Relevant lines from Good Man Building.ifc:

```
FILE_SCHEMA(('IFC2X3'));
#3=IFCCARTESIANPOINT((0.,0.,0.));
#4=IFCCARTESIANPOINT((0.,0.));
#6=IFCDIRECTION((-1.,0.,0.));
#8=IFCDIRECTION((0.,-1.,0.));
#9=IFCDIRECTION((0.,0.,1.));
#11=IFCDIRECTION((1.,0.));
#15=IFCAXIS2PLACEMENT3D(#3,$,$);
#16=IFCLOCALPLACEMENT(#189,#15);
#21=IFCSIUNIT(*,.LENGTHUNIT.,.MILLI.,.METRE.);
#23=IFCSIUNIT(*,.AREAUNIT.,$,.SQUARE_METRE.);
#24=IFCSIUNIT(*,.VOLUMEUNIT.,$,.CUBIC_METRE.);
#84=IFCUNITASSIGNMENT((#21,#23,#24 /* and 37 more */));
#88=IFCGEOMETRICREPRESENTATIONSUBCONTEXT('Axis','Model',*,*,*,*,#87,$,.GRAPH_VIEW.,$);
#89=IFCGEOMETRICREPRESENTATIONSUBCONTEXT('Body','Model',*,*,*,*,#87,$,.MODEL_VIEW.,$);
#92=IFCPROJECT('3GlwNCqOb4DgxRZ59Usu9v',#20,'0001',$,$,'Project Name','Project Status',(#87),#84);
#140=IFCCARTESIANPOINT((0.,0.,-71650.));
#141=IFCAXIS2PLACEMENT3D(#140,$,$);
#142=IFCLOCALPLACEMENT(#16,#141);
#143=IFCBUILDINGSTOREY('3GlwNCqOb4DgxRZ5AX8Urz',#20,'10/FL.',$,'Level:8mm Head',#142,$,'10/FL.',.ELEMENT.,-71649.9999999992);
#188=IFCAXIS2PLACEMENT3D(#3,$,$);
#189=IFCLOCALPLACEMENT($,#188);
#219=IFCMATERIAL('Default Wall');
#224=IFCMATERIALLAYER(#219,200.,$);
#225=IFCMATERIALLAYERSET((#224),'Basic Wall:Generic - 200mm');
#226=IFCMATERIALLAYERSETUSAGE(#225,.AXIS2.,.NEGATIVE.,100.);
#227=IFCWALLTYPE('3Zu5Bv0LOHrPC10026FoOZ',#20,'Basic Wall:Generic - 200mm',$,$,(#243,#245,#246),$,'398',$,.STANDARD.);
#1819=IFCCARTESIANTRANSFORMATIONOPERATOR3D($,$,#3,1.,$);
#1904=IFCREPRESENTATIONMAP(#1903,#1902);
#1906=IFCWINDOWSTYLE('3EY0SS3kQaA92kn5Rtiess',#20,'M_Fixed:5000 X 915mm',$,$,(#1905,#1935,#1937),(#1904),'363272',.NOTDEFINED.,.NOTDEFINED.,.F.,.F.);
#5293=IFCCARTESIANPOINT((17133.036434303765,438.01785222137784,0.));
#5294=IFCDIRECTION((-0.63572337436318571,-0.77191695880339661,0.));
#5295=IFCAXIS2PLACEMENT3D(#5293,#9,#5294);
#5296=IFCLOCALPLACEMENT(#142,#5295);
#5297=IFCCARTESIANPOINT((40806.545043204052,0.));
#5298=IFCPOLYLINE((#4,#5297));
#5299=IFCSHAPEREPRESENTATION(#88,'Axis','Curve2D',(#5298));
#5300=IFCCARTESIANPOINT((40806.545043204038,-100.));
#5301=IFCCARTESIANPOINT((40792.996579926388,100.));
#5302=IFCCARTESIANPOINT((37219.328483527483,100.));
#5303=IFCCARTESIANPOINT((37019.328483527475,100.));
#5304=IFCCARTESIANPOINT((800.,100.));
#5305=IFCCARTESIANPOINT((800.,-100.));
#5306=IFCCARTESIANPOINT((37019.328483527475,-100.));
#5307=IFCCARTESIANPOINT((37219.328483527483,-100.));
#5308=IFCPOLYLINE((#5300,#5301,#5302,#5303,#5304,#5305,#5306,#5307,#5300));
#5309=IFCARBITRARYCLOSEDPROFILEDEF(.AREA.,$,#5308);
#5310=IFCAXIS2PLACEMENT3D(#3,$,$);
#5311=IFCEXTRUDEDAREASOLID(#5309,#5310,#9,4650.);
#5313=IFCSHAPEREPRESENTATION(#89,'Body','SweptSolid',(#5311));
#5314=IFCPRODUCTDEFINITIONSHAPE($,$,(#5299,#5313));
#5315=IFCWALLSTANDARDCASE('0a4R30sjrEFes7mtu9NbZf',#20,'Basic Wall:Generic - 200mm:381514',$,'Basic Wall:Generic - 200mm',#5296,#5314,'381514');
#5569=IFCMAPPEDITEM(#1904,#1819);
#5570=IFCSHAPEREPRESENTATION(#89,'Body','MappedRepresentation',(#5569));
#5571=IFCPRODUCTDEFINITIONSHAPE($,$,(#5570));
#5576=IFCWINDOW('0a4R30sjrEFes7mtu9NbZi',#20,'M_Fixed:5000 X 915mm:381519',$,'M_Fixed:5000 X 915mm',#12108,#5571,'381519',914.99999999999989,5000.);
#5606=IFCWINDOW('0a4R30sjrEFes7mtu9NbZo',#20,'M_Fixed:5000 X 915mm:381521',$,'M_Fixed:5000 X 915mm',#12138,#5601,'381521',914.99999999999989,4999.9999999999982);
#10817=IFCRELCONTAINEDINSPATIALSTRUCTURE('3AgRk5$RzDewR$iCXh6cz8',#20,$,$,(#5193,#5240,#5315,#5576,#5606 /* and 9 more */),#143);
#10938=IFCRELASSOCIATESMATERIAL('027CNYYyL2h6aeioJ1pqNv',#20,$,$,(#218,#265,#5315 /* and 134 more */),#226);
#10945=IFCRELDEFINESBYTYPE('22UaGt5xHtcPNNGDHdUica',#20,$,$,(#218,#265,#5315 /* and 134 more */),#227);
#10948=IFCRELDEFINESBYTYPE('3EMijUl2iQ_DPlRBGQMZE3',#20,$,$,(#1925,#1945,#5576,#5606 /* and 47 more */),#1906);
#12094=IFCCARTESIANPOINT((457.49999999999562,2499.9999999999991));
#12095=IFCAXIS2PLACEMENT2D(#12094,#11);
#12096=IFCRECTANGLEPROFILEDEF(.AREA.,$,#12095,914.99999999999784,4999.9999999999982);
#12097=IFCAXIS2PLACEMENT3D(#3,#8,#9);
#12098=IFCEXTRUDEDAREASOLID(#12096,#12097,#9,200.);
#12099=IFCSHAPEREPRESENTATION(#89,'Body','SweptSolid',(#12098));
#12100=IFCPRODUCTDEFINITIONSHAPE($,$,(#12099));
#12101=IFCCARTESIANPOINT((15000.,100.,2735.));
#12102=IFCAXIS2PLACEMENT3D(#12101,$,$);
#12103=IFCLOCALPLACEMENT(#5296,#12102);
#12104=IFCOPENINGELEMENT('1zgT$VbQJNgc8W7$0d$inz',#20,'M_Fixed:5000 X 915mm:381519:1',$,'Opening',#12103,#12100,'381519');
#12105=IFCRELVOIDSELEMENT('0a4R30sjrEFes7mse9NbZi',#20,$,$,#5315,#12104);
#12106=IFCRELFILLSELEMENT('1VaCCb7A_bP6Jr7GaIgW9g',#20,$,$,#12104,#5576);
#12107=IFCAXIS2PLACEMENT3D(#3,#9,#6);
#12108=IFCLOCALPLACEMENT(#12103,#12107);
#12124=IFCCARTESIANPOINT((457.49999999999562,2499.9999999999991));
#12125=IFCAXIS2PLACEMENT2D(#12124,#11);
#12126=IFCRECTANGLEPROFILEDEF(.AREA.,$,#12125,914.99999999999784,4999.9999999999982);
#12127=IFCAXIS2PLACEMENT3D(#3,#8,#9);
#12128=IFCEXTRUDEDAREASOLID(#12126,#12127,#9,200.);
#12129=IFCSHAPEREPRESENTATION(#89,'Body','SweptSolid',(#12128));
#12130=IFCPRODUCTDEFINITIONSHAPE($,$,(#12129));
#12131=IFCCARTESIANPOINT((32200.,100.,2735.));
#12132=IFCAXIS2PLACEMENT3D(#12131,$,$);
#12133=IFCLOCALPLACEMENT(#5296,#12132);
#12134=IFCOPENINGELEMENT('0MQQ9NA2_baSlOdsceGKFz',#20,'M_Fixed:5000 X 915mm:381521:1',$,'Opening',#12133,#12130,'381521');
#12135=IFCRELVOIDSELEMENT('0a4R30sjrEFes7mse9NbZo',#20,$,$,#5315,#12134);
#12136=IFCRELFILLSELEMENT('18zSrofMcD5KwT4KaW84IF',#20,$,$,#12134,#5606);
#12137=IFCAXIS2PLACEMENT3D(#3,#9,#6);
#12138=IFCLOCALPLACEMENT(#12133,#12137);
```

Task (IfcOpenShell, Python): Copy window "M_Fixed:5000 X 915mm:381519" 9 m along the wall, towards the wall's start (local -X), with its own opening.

```python
import ifcopenshell
import ifcopenshell.api.feature
import ifcopenshell.api.geometry
import ifcopenshell.api.root
import ifcopenshell.geom
import ifcopenshell.util.element
import ifcopenshell.util.placement
import ifcopenshell.util.shape
import ifcopenshell.util.unit

model = ifcopenshell.open("Good Man Building.ifc")
unit_scale = ifcopenshell.util.unit.calculate_unit_scale(model)
settings = ifcopenshell.geom.settings()


def volume(element):
    """Net volume in cubic metres, openings subtracted."""
    shape = ifcopenshell.geom.create_shape(settings, element)
    return ifcopenshell.util.shape.get_volume(shape.geometry)


def reuse_history(source, copy):
    """copy_class also copies each property set's owner history, people and application; keep the originals."""
    for rel in copy.IsDefinedBy:
        if rel.is_a("IfcRelDefinesByProperties") and (history := rel.RelatingPropertyDefinition.OwnerHistory):
            rel.RelatingPropertyDefinition.OwnerHistory = source.OwnerHistory
            ifcopenshell.util.element.remove_deep2(model, history)


window = model.by_id(5576)
opening = window.FillsVoids[0].RelatingOpeningElement
wall = opening.VoidsElements[0].RelatingBuildingElement
before = volume(wall)
shift = ifcopenshell.util.placement.get_local_placement(wall.ObjectPlacement)[:3, 0] * -9 / unit_scale

# copy_class copies the void relationship, type, container and properties, but no geometry.
new_opening = ifcopenshell.api.root.copy_class(model, product=opening)
new_opening.Representation = ifcopenshell.util.element.copy_deep(
    model, opening.Representation, exclude=["IfcGeometricRepresentationContext", "IfcRepresentationMap"]
)
new_opening.Name = "M_Fixed:5000 X 915mm"
new_opening.Tag = None
new_window = ifcopenshell.api.root.copy_class(model, product=window)
new_window.Representation = ifcopenshell.util.element.copy_deep(
    model, window.Representation, exclude=["IfcGeometricRepresentationContext", "IfcRepresentationMap"]
)
new_window.Name = "M_Fixed:5000 X 915mm"
new_window.Tag = None
reuse_history(window, new_window)
fills = ifcopenshell.api.feature.add_filling(model, opening=new_opening, element=new_window)
fills.OwnerHistory = new_window.OwnerHistory  # required in IFC2X3

for old, new in ((opening, new_opening), (window, new_window)):
    matrix = ifcopenshell.util.placement.get_local_placement(old.ObjectPlacement)
    matrix[:3, 3] += shift
    ifcopenshell.api.geometry.edit_object_placement(model, product=new, matrix=matrix, is_si=False)

after = volume(wall)

print(f"wall volume {before:.3f} -> {after:.3f} m3")

model.write("Good Man Building_updated.ifc")
```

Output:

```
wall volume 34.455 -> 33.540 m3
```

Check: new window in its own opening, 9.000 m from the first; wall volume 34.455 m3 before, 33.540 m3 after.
